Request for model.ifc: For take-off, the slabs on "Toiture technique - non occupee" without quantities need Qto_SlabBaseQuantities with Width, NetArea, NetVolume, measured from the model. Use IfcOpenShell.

First a look at what the model holds.

```python
import ifcopenshell
import ifcopenshell.util.element
import ifcopenshell.util.unit

model = ifcopenshell.open("model.ifc")
print(model.schema)
for unit_type in ("LENGTHUNIT", "AREAUNIT", "VOLUMEUNIT"):
    print(unit_type, ifcopenshell.util.unit.calculate_unit_scale(model, unit_type))
storey = next(s for s in model.by_type("IfcBuildingStorey") if s.Name == "Toiture technique - non occupee")
slabs = [e for e in ifcopenshell.util.element.get_decomposition(storey) if e.is_a("IfcSlab")]
for e in sorted(slabs, key=lambda e: e.id()):
    print(e.id(), e.is_a(), e.Name, list(ifcopenshell.util.element.get_psets(e, qtos_only=True)), sep=" | ")
```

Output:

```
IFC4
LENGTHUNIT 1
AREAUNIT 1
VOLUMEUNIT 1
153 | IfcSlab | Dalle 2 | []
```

```python
import ifcopenshell
import ifcopenshell.api.pset
import ifcopenshell.geom
import ifcopenshell.util.element
import ifcopenshell.util.shape
import ifcopenshell.util.unit

model = ifcopenshell.open("model.ifc")
unit_scale = ifcopenshell.util.unit.calculate_unit_scale(model)
area_scale = ifcopenshell.util.unit.calculate_unit_scale(model, "AREAUNIT")
volume_scale = ifcopenshell.util.unit.calculate_unit_scale(model, "VOLUMEUNIT")
settings = ifcopenshell.geom.settings()

storey = next(s for s in model.by_type("IfcBuildingStorey") if s.Name == "Toiture technique - non occupee")
slabs = [e for e in ifcopenshell.util.element.get_decomposition(storey) if e.is_a("IfcSlab")]

for e in sorted(slabs, key=lambda e: e.id()):
    if ifcopenshell.util.element.get_psets(e, qtos_only=True, should_inherit=False):
        continue
    # Geometry comes back in metres, in the element's own axes.
    shape = ifcopenshell.geom.create_shape(settings, e)
    values = {
        "Width": ifcopenshell.util.shape.get_z(shape.geometry) / unit_scale,
        "NetArea": ifcopenshell.util.shape.get_footprint_area(shape.geometry) / area_scale,
        "NetVolume": ifcopenshell.util.shape.get_volume(shape.geometry) / volume_scale,
    }
    qto = ifcopenshell.api.pset.add_qto(model, product=e, name="Qto_SlabBaseQuantities")
    ifcopenshell.api.pset.edit_qto(model, qto=qto, properties=values)
    print(e.id(), {k: round(v, 3) for k, v in values.items()})

model.write("model_updated.ifc")
```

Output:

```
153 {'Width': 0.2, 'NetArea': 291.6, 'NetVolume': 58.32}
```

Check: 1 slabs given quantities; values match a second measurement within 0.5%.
